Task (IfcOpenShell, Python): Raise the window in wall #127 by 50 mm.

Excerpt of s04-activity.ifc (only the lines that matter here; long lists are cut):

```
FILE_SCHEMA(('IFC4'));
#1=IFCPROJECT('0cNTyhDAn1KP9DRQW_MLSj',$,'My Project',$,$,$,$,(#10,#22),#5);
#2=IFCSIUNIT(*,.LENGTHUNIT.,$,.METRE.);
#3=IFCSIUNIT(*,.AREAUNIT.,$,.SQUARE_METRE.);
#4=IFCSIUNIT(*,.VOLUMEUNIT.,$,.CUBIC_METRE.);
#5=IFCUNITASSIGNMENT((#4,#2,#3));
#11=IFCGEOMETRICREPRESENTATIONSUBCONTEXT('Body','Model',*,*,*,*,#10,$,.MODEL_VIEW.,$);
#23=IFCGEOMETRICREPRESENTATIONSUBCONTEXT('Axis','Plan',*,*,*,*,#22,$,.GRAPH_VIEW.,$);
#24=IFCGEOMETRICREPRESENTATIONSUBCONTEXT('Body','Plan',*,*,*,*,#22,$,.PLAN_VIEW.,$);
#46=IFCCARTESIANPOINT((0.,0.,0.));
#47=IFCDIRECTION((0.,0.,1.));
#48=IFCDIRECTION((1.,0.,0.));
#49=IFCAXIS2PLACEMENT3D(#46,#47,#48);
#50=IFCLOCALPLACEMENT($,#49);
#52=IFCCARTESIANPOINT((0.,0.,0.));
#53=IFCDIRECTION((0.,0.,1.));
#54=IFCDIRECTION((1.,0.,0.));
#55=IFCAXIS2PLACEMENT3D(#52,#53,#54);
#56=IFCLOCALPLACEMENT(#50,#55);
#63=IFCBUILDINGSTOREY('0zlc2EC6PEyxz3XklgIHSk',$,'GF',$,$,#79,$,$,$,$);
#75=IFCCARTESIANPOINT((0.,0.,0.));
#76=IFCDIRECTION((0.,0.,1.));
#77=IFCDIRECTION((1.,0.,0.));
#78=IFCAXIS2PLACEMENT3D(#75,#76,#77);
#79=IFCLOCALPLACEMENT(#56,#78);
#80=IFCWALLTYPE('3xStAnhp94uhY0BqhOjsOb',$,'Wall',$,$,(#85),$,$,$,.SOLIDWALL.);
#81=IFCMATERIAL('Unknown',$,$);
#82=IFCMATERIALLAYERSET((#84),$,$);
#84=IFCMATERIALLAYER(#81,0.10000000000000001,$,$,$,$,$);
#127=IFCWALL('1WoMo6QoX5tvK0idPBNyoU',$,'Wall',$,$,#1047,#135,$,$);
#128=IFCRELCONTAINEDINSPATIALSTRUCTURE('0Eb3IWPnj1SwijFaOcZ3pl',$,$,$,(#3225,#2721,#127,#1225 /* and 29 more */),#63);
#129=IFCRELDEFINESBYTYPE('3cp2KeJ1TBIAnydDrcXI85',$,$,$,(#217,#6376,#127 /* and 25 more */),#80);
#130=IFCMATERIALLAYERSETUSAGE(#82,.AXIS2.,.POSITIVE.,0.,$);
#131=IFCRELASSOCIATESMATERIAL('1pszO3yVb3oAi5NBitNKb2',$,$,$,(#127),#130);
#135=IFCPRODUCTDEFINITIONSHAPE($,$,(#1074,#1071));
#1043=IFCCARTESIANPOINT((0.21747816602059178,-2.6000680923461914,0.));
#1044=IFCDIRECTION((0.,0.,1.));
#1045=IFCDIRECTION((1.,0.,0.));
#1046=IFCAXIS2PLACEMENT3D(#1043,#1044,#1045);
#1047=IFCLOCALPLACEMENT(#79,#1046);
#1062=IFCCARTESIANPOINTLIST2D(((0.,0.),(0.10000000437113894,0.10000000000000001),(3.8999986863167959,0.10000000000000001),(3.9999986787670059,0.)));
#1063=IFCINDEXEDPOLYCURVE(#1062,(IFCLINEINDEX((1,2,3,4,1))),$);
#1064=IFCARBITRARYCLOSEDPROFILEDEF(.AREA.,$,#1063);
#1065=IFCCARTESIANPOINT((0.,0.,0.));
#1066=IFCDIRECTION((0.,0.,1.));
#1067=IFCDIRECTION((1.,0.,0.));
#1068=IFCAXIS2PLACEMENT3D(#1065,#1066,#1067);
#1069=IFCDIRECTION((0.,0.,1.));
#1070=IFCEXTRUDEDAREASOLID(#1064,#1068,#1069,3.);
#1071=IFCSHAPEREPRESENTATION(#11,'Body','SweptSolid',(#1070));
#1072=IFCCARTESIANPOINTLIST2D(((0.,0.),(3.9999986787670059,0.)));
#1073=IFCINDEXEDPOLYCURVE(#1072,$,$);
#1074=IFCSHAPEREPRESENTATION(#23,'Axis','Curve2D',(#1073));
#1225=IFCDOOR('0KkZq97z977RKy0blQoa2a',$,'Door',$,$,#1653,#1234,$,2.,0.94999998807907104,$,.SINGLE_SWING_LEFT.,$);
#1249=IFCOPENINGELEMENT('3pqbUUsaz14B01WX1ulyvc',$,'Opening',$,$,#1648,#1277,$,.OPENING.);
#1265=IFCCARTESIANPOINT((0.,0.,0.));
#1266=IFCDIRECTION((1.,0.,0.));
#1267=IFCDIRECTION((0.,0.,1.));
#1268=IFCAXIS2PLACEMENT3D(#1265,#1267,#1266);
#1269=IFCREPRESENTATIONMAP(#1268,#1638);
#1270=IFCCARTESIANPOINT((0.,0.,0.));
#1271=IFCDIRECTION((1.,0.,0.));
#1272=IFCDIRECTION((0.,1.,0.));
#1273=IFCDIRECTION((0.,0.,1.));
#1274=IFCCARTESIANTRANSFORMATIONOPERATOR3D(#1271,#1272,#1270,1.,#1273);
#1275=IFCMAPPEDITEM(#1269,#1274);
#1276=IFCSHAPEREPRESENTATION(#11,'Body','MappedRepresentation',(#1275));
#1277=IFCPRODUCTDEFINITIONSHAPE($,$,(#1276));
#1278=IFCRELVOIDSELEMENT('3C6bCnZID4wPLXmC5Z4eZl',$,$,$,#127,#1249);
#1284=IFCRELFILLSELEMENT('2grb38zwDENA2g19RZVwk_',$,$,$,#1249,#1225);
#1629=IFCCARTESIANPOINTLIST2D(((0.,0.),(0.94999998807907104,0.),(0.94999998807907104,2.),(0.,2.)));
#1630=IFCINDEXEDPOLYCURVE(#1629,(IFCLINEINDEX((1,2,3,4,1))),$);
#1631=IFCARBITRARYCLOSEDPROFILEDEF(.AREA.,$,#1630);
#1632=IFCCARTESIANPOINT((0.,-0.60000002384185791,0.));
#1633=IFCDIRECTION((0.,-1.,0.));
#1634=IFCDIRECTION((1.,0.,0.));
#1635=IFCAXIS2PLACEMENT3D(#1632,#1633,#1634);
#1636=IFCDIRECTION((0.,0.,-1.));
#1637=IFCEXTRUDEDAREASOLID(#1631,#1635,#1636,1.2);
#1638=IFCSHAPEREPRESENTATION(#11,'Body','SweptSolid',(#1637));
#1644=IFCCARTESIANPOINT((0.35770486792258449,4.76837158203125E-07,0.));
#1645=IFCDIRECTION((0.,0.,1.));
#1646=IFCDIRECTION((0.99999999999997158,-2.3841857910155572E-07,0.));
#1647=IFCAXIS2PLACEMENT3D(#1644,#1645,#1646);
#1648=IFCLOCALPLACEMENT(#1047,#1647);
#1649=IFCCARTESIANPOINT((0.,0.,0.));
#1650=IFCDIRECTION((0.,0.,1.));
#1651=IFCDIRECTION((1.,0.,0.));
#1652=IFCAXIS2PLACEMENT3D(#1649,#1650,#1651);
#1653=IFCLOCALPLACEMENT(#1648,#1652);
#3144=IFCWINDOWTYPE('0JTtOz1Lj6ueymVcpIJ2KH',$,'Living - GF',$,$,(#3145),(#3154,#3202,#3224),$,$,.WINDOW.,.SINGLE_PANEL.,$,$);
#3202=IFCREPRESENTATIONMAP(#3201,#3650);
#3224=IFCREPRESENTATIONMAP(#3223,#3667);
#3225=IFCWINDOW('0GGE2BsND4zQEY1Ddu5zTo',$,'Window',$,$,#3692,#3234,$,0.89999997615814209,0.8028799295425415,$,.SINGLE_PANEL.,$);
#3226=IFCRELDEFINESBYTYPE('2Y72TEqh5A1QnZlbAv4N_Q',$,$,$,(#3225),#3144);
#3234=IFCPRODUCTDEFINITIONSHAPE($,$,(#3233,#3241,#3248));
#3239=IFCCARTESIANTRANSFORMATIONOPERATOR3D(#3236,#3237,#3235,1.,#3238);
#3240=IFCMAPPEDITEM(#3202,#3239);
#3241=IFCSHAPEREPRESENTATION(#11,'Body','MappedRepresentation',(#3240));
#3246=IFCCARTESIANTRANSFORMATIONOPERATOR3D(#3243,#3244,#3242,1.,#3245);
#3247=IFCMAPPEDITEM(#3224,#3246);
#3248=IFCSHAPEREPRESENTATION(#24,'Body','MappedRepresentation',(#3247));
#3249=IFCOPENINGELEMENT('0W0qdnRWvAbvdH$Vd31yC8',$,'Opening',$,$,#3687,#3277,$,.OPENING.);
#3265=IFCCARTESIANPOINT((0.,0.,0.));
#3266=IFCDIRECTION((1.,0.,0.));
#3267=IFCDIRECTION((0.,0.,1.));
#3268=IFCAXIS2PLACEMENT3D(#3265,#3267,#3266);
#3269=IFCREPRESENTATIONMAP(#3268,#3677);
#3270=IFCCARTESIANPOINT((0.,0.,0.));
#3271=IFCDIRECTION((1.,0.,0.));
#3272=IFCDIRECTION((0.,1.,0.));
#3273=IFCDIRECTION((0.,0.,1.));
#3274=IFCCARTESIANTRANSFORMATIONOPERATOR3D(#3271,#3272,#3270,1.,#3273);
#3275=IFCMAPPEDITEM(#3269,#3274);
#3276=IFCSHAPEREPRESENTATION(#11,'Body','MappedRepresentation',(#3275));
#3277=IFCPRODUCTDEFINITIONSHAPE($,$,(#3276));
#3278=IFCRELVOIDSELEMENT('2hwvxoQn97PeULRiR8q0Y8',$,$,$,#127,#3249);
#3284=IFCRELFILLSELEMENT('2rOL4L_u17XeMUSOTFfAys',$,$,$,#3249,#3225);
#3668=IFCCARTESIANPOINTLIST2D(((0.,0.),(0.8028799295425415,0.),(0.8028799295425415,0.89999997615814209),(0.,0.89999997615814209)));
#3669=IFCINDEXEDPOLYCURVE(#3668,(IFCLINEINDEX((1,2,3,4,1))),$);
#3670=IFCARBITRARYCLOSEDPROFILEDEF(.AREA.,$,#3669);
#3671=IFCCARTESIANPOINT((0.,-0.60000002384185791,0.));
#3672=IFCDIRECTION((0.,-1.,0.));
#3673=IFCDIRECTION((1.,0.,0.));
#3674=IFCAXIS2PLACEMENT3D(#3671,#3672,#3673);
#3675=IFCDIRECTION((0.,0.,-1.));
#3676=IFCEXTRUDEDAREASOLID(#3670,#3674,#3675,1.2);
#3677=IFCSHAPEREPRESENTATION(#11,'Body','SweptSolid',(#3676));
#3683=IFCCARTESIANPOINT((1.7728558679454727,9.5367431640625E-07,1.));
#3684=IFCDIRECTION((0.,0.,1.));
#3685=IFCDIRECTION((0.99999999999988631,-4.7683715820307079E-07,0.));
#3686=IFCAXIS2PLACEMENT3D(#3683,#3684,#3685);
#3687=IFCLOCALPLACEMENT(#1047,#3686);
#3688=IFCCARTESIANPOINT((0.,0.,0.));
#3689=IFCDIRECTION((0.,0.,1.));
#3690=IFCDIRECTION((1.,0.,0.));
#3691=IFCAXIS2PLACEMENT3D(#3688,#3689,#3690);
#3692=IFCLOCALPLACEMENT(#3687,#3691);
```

```python
import numpy as np
import ifcopenshell
import ifcopenshell.api.geometry
import ifcopenshell.util.placement
import ifcopenshell.util.unit

model = ifcopenshell.open("s04-activity.ifc")
unit_scale = ifcopenshell.util.unit.calculate_unit_scale(model)

window = model.by_guid("0GGE2BsND4zQEY1Ddu5zTo")
opening = window.FillsVoids[0].RelatingOpeningElement
dz = 0.05 / unit_scale

shift = np.array([0.0, 0.0, dz])
# The window is placed relative to its opening, so it follows when the opening moves.
matrix = ifcopenshell.util.placement.get_local_placement(opening.ObjectPlacement)
matrix[:3, 3] += shift
ifcopenshell.api.geometry.edit_object_placement(
    model, product=opening, matrix=matrix, is_si=False, should_transform_children=True
)

print(f"moved by {dz * unit_scale:+.3f} m")

model.write("s04-activity_rev.ifc")
```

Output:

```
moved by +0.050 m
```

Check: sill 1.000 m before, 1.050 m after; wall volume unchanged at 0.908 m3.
